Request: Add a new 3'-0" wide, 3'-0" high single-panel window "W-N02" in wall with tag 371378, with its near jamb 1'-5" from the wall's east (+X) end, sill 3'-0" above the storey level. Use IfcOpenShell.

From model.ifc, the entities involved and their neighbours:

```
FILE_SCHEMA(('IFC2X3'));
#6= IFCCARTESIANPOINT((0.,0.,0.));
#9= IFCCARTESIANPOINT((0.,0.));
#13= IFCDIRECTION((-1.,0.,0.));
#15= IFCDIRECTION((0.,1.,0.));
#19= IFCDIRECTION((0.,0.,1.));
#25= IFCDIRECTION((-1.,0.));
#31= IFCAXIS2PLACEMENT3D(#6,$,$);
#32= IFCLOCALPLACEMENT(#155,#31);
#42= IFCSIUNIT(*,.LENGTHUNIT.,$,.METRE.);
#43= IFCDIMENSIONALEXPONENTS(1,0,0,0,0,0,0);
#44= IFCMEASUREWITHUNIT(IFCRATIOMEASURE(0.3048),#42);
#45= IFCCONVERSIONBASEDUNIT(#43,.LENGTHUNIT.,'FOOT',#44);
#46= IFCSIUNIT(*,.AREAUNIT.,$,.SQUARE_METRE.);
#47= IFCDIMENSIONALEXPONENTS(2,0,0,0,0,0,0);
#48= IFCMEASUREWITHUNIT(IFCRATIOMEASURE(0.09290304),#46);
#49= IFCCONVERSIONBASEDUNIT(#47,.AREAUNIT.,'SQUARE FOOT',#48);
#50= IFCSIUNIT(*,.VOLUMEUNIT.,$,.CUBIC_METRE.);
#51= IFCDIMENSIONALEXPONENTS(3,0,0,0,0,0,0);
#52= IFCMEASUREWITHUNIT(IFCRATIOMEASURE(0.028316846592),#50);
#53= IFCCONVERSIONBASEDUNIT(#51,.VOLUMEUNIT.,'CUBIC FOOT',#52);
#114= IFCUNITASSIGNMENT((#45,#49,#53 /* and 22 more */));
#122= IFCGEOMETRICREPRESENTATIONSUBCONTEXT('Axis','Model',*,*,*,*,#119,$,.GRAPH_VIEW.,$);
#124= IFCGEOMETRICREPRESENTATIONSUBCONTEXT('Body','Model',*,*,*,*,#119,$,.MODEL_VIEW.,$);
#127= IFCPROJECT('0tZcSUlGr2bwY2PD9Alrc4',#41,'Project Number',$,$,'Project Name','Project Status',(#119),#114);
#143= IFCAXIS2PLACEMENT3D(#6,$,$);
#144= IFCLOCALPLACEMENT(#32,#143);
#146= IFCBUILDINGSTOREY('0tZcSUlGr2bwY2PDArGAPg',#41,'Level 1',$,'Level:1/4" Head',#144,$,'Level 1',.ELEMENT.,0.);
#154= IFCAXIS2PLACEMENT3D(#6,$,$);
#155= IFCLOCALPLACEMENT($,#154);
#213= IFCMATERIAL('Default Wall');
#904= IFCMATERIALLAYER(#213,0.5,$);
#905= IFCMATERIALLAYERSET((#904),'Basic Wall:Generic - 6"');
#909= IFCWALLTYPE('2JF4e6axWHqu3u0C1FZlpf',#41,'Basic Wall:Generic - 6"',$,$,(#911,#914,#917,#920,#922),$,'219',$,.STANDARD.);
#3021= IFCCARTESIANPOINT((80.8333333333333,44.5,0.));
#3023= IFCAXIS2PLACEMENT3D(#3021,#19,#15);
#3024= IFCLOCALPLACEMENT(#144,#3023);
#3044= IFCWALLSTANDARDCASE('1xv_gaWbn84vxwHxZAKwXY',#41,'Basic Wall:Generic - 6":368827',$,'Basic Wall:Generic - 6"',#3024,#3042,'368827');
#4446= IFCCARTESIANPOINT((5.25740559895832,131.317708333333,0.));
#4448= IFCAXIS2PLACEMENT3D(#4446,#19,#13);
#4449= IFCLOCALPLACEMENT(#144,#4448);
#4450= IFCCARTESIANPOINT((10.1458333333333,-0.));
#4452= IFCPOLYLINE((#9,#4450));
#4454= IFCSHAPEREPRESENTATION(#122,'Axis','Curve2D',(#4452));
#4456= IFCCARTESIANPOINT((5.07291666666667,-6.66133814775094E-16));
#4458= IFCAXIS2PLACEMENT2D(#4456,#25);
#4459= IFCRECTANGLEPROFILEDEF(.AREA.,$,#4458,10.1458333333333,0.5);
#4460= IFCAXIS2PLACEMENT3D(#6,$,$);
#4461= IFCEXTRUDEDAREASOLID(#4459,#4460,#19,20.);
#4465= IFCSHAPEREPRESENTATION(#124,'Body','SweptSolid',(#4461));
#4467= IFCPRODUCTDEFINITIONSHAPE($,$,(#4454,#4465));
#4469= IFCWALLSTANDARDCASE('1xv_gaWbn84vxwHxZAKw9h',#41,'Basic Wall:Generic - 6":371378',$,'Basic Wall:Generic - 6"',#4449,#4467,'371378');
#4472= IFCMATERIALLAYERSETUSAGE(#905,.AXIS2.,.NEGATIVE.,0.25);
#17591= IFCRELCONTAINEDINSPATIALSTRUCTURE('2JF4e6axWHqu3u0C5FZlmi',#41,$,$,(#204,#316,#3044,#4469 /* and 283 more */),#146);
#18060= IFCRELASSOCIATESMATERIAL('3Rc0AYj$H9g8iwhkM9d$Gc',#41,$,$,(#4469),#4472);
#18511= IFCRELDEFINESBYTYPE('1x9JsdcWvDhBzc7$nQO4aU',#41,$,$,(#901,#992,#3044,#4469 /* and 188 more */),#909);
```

```python
import numpy as np
import ifcopenshell
import ifcopenshell.api.feature
import ifcopenshell.api.geometry
import ifcopenshell.api.root
import ifcopenshell.api.spatial
import ifcopenshell.api.type
import ifcopenshell.geom
import ifcopenshell.util.element
import ifcopenshell.util.placement
import ifcopenshell.util.representation
import ifcopenshell.util.shape
import ifcopenshell.util.unit

model = ifcopenshell.open("model.ifc")
unit_scale = ifcopenshell.util.unit.calculate_unit_scale(model)
settings = ifcopenshell.geom.settings()


def volume(element):
    """Net volume in cubic metres, openings subtracted."""
    shape = ifcopenshell.geom.create_shape(settings, element)
    return ifcopenshell.util.shape.get_volume(shape.geometry)


wall = model.by_id(4469)
storey = ifcopenshell.util.element.get_container(wall, ifc_class="IfcBuildingStorey")
context = ifcopenshell.util.representation.get_context(model, "Model", "Body", "MODEL_VIEW")
before = volume(wall)

width, height, from_end, sill = 0.9144, 0.9144, 0.4318, 0.9144  # metres

# The wall runs along its own X axis, and the end named is its -X end.
wall_shape = ifcopenshell.geom.create_shape(settings, wall)
x, y, z = ifcopenshell.util.shape.get_vertices(wall_shape.geometry).T
start = x.min() + from_end
face, thickness = float(y.min()), float(y.max() - y.min())
wall_matrix = ifcopenshell.util.placement.get_local_placement(wall.ObjectPlacement)
level = ifcopenshell.util.placement.get_local_placement(storey.ObjectPlacement)[2, 3]


def in_wall(x, y):
    """Placement at x, y metres in the wall's axes, at sill height."""
    matrix = wall_matrix.copy()
    matrix[:, 3] = wall_matrix @ np.array([x / unit_scale, y / unit_scale, 0.0, 1.0])
    matrix[2, 3] = level + sill / unit_scale
    return matrix


# Opening: a box that overshoots both wall faces by 50 mm.
opening = ifcopenshell.api.root.create_entity(model, ifc_class="IfcOpeningElement")
box = ifcopenshell.api.geometry.add_wall_representation(
    model, context=context, length=width, height=height, thickness=thickness + 0.1
)
ifcopenshell.api.geometry.assign_representation(model, product=opening, representation=box)
ifcopenshell.api.geometry.edit_object_placement(model, product=opening, matrix=in_wall(start, face - 0.05), is_si=False)
ifcopenshell.api.feature.add_feature(model, feature=opening, element=wall)

window = ifcopenshell.api.root.create_entity(model, ifc_class="IfcWindow", name="W-N02")
window.OverallWidth, window.OverallHeight = width / unit_scale, height / unit_scale
body = ifcopenshell.api.geometry.add_window_representation(
    model,
    context=context,
    overall_width=window.OverallWidth,
    overall_height=window.OverallHeight,
    partition_type="SINGLE_PANEL",
)
ifcopenshell.api.geometry.assign_representation(model, product=window, representation=body)
ifcopenshell.api.spatial.assign_container(model, products=[window], relating_structure=storey)
fills = ifcopenshell.api.feature.add_filling(model, opening=opening, element=window)
fills.OwnerHistory = window.OwnerHistory  # required in IFC2X3

# IFC2X3 keeps the operation on the window style.
style = ifcopenshell.api.root.create_entity(model, ifc_class="IfcWindowStyle", name="W-N02")
style.OperationType, style.ConstructionType = "SINGLE_PANEL", "NOTDEFINED"
style.ParameterTakesPrecedence = style.Sizeable = False
ifcopenshell.api.type.assign_type(model, related_objects=[window], relating_type=style)

# Centre the window in the wall's thickness.
ifcopenshell.api.geometry.edit_object_placement(model, product=window, matrix=in_wall(start, face), is_si=False)
window_shape = ifcopenshell.geom.create_shape(settings, window)
depth = ifcopenshell.util.shape.get_vertices(window_shape.geometry)[:, 1]
offset = face + thickness / 2 - (depth.min() + depth.max()) / 2
ifcopenshell.api.geometry.edit_object_placement(model, product=window, matrix=in_wall(start, offset), is_si=False)

after = volume(wall)

print(f"wall volume {before:.3f} -> {after:.3f} m3")

model.write("model_v2.ifc")
```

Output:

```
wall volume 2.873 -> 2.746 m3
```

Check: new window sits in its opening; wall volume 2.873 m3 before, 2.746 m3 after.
